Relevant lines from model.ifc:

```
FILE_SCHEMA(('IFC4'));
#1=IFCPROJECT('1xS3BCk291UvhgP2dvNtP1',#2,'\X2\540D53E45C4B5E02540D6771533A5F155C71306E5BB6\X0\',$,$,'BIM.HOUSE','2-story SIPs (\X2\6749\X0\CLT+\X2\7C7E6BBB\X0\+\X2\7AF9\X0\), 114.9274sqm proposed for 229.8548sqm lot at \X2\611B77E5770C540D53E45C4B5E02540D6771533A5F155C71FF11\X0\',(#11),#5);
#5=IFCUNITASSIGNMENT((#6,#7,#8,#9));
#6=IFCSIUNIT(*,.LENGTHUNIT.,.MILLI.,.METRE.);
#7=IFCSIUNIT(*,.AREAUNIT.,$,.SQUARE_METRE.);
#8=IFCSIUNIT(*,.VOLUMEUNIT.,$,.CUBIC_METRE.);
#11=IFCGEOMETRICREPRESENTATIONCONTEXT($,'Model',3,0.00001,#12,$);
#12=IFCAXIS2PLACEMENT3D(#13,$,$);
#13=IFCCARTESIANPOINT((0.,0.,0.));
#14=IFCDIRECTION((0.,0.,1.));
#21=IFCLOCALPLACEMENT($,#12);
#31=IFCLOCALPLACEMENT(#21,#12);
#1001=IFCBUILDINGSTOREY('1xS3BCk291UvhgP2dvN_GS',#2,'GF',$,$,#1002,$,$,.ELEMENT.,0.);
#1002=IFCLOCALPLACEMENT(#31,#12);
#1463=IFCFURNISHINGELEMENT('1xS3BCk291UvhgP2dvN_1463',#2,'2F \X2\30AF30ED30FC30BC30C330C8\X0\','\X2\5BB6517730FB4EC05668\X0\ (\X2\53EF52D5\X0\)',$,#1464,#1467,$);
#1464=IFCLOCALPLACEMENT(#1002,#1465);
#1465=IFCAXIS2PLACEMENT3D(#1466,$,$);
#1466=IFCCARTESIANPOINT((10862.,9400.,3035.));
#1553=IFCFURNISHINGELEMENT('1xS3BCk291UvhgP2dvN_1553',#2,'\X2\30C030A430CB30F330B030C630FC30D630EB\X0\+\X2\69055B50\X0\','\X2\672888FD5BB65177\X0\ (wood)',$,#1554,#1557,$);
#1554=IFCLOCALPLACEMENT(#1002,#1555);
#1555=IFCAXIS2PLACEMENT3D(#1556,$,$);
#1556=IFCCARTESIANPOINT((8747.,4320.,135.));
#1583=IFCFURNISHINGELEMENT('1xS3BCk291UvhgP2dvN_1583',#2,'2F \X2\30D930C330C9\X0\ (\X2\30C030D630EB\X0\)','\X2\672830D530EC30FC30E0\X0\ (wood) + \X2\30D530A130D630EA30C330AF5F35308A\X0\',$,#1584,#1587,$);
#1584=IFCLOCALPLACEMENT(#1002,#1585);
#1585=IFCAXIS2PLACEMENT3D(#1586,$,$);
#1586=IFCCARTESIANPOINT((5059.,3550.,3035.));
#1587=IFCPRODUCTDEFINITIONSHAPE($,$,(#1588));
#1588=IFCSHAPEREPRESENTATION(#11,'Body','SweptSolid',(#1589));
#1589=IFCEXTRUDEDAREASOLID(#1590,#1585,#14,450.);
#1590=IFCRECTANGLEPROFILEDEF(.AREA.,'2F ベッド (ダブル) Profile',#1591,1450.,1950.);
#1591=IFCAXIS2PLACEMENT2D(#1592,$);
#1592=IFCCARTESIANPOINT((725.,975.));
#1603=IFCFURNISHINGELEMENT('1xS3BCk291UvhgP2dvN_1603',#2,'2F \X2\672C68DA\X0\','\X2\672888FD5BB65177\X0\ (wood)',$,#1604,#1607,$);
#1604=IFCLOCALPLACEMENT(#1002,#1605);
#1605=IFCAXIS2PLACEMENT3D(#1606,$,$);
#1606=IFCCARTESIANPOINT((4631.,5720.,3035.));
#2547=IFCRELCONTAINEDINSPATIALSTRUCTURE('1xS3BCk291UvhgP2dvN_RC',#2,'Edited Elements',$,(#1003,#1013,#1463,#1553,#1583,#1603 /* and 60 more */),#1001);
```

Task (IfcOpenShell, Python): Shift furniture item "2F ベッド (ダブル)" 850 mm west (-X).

```python
import ifcopenshell
import ifcopenshell.api.geometry
import ifcopenshell.util.placement
import ifcopenshell.util.unit

model = ifcopenshell.open("model.ifc")
unit_scale = ifcopenshell.util.unit.calculate_unit_scale(model)

item = model.by_guid("1xS3BCk291UvhgP2dvN_1583")
matrix = ifcopenshell.util.placement.get_local_placement(item.ObjectPlacement)
matrix[0, 3] -= 0.85 / unit_scale
ifcopenshell.api.geometry.edit_object_placement(model, product=item, matrix=matrix, is_si=False)

print(ifcopenshell.util.placement.get_local_placement(item.ObjectPlacement).round(3) + 0.0)

model.write("model-out.ifc")
```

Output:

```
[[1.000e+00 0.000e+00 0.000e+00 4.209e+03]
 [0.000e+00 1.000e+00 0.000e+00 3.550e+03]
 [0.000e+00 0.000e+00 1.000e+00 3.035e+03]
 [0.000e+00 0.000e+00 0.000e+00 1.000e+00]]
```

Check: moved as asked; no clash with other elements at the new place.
